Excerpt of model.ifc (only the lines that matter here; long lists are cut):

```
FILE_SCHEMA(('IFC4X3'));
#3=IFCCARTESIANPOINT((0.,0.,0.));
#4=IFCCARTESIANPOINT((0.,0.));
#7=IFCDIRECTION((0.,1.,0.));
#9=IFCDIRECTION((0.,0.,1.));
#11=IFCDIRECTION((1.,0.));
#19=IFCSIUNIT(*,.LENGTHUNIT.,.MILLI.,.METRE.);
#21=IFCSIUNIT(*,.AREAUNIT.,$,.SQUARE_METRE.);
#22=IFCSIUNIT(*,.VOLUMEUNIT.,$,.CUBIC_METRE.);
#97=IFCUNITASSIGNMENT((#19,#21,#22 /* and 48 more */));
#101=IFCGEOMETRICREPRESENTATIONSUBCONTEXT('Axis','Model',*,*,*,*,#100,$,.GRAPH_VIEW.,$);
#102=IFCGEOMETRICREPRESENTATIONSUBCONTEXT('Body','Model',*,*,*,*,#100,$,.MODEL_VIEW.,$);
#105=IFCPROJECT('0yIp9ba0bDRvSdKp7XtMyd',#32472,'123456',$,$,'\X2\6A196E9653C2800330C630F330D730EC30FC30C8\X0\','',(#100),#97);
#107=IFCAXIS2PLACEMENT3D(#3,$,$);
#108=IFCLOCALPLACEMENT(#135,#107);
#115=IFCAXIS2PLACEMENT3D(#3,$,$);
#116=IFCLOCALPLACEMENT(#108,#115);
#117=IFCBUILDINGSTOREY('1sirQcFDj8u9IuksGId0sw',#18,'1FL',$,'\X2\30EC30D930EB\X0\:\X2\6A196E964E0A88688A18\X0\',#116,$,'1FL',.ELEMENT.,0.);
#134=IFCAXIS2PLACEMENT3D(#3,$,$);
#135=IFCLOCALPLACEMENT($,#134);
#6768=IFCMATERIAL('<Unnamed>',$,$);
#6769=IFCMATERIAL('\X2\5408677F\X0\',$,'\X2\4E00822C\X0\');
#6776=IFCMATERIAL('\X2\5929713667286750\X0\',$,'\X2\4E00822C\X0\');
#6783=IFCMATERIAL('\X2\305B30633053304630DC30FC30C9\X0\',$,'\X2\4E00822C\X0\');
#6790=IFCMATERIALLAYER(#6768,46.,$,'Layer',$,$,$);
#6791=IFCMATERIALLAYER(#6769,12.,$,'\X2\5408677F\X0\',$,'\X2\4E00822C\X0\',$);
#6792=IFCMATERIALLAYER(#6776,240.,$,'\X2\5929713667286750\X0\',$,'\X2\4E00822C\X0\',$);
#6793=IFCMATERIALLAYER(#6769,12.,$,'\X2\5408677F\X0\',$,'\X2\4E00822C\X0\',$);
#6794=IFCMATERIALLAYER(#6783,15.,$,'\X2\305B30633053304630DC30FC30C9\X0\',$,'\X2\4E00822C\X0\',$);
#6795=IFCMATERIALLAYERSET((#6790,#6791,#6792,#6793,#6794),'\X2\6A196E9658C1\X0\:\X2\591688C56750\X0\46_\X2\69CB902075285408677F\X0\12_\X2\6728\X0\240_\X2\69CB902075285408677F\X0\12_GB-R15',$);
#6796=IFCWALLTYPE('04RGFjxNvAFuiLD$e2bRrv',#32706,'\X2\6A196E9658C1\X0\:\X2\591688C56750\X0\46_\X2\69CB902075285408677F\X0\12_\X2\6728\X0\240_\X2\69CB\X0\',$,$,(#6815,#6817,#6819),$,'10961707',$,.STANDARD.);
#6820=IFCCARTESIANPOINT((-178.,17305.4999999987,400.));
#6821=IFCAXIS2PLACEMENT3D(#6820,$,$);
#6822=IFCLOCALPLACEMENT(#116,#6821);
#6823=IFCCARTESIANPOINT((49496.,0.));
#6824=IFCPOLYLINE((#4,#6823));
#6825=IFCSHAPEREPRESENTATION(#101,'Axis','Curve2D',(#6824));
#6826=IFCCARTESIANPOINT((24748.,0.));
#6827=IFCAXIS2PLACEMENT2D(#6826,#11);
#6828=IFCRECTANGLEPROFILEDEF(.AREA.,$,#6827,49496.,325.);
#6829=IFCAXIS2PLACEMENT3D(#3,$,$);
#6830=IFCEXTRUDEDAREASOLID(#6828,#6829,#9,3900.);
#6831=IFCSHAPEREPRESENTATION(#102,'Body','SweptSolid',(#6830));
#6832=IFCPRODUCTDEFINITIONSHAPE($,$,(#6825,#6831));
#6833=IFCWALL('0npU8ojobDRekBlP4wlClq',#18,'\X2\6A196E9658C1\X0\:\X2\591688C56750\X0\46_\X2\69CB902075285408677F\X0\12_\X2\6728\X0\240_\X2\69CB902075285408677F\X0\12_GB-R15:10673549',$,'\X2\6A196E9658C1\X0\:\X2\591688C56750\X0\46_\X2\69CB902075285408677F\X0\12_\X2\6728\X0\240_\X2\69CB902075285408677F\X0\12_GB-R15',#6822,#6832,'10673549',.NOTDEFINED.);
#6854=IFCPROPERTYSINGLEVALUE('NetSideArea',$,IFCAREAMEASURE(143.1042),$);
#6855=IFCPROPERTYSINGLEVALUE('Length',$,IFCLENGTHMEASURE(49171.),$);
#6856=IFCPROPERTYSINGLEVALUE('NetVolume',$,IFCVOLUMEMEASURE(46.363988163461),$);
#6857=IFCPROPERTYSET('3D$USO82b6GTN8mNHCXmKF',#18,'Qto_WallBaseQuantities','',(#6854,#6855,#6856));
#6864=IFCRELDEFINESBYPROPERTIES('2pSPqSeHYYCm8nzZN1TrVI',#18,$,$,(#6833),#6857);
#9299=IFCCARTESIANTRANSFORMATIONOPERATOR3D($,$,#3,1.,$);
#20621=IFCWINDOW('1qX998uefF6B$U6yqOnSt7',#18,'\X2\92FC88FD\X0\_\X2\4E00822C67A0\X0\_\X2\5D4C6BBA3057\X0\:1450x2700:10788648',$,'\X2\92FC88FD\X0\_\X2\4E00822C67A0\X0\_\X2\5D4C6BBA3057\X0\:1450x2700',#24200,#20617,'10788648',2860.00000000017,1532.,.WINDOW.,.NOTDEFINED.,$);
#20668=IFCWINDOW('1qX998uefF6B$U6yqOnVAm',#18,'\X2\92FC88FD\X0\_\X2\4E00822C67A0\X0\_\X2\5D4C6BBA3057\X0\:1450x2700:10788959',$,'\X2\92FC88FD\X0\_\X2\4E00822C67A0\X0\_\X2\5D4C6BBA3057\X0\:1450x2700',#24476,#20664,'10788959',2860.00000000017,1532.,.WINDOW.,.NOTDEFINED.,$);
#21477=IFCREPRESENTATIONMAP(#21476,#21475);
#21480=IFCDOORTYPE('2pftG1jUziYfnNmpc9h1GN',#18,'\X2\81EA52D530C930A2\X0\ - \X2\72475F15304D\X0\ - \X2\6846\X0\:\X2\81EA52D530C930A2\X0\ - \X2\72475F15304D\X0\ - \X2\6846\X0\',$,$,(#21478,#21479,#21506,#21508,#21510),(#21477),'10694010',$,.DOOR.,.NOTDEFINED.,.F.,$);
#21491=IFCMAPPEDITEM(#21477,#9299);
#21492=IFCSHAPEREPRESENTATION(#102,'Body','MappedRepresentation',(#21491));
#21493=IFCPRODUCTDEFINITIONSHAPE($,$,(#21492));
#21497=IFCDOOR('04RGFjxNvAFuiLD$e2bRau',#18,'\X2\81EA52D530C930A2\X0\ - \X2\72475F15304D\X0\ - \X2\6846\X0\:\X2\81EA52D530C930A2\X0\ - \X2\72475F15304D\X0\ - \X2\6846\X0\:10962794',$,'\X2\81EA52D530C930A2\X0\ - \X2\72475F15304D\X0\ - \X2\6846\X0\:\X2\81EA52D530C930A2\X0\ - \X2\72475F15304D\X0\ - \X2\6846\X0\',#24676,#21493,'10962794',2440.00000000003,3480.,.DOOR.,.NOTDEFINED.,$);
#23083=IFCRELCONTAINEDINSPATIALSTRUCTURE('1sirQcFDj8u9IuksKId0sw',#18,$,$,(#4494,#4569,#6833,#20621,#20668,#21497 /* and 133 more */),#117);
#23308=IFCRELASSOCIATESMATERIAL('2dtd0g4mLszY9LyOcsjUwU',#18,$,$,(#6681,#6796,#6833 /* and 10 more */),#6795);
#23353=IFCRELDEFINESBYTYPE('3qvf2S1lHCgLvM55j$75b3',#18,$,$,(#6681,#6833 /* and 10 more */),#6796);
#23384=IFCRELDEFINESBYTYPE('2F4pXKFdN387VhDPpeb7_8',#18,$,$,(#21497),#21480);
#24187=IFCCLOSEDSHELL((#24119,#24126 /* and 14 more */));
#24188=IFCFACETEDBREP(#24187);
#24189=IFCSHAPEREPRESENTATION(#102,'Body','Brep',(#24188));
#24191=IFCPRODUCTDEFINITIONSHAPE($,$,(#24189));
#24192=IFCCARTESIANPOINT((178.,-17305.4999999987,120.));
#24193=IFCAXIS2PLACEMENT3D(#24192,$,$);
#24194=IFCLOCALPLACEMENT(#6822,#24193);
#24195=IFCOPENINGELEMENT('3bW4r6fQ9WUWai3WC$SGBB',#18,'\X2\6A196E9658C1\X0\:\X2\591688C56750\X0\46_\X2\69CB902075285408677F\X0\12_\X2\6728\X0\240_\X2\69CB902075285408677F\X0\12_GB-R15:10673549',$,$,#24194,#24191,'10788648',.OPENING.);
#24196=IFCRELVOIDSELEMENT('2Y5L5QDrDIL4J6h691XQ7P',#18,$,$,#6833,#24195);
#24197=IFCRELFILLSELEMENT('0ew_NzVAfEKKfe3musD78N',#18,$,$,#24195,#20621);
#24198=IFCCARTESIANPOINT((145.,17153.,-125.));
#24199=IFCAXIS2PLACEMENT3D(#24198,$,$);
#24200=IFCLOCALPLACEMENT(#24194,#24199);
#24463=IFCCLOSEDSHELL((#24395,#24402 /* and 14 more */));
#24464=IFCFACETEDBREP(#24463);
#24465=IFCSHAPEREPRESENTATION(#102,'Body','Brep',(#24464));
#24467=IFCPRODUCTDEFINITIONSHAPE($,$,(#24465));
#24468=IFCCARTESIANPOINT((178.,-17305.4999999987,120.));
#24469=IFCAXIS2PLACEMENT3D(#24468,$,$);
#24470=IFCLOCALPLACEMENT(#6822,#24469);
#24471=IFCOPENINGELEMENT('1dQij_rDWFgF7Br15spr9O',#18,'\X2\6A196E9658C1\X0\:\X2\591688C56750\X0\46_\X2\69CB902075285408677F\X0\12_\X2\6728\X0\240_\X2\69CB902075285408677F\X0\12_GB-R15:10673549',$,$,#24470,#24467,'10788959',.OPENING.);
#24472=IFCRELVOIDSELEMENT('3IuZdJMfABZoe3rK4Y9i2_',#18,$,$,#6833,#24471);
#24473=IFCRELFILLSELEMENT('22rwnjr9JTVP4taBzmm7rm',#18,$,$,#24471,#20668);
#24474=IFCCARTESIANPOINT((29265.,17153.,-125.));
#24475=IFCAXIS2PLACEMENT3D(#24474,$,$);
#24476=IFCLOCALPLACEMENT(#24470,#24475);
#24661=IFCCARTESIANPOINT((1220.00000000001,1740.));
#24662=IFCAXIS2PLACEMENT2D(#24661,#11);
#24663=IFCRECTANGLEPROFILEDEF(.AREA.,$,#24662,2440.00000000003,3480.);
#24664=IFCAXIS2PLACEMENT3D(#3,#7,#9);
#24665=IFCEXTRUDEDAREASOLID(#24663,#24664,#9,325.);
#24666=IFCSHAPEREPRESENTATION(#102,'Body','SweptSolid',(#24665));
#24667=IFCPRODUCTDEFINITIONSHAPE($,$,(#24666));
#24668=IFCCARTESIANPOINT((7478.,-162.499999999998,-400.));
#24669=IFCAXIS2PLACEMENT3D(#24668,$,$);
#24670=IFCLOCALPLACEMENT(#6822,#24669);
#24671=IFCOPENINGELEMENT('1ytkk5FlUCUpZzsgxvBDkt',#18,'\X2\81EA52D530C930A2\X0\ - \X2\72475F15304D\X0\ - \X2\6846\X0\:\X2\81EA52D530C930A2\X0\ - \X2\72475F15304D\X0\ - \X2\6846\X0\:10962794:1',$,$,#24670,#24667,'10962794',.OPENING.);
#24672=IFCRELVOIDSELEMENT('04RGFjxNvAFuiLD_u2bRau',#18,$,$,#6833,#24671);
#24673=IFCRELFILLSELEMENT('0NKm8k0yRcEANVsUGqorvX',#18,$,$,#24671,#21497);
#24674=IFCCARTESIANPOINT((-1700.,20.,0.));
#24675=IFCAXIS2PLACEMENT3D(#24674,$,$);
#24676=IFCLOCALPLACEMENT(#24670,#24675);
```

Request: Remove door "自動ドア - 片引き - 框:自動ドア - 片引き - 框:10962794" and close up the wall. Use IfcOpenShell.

```python
import ifcopenshell
import ifcopenshell.api.feature
import ifcopenshell.api.pset
import ifcopenshell.api.root
import ifcopenshell.geom
import ifcopenshell.util.element
import ifcopenshell.util.shape
import ifcopenshell.util.unit

model = ifcopenshell.open("model.ifc")
area_scale = ifcopenshell.util.unit.calculate_unit_scale(model, "AREAUNIT")
volume_scale = ifcopenshell.util.unit.calculate_unit_scale(model, "VOLUMEUNIT")
settings = ifcopenshell.geom.settings()


def volume(element):
    """Net volume in cubic metres, openings subtracted."""
    shape = ifcopenshell.geom.create_shape(settings, element)
    return ifcopenshell.util.shape.get_volume(shape.geometry)


door = model.by_guid("04RGFjxNvAFuiLD$e2bRau")
opening = door.FillsVoids[0].RelatingOpeningElement
wall = opening.VoidsElements[0].RelatingBuildingElement
before = volume(wall)

ifcopenshell.api.root.remove_product(model, product=door)
ifcopenshell.api.feature.remove_feature(model, feature=opening)

after = volume(wall)
thickness = 0.325  # wall thickness in metres

# Update the wall's stored quantities.
pset = model.by_id(ifcopenshell.util.element.get_pset(wall, "Qto_WallBaseQuantities", should_inherit=False)["id"])
ifcopenshell.api.pset.edit_pset(model, pset=pset, properties={
    "NetSideArea": model.create_entity("IfcAreaMeasure", after / thickness / area_scale),
    "NetVolume": model.create_entity("IfcVolumeMeasure", after / volume_scale),
})

print(f"wall volume {before:.3f} -> {after:.3f} m3")

model.write("model_rev.ifc")
```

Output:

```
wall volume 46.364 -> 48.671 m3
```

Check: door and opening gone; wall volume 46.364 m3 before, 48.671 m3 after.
